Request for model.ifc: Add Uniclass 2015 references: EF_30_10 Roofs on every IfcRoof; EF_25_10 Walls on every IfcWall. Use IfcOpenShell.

First a look at what the model holds.

```python
import ifcopenshell

model = ifcopenshell.open("model.ifc")
print(model.schema)
print("classifications:", [c.Name for c in model.by_type("IfcClassification")])
for ifc_class in ("IfcDoor", "IfcRoof", "IfcStair", "IfcWall", "IfcWindow"):
    print(ifc_class, len(model.by_type(ifc_class)))
```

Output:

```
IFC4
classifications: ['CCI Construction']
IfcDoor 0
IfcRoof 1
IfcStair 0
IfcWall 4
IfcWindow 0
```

```python
import ifcopenshell
import ifcopenshell.api.classification

model = ifcopenshell.open("model.ifc")

system = ifcopenshell.api.classification.add_classification(model, classification="Uniclass 2015")

codes = {
    "IfcRoof": ("EF_30_10", "Roofs"),
    "IfcWall": ("EF_25_10", "Walls"),
}
for ifc_class, (code, name) in codes.items():
    products = model.by_type(ifc_class)
    ifcopenshell.api.classification.add_reference(
        model, products=products, classification=system, identification=code, name=name
    )
    print(code, len(products))

model.write("model_v2.ifc")
```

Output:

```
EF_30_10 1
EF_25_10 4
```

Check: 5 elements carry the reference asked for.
